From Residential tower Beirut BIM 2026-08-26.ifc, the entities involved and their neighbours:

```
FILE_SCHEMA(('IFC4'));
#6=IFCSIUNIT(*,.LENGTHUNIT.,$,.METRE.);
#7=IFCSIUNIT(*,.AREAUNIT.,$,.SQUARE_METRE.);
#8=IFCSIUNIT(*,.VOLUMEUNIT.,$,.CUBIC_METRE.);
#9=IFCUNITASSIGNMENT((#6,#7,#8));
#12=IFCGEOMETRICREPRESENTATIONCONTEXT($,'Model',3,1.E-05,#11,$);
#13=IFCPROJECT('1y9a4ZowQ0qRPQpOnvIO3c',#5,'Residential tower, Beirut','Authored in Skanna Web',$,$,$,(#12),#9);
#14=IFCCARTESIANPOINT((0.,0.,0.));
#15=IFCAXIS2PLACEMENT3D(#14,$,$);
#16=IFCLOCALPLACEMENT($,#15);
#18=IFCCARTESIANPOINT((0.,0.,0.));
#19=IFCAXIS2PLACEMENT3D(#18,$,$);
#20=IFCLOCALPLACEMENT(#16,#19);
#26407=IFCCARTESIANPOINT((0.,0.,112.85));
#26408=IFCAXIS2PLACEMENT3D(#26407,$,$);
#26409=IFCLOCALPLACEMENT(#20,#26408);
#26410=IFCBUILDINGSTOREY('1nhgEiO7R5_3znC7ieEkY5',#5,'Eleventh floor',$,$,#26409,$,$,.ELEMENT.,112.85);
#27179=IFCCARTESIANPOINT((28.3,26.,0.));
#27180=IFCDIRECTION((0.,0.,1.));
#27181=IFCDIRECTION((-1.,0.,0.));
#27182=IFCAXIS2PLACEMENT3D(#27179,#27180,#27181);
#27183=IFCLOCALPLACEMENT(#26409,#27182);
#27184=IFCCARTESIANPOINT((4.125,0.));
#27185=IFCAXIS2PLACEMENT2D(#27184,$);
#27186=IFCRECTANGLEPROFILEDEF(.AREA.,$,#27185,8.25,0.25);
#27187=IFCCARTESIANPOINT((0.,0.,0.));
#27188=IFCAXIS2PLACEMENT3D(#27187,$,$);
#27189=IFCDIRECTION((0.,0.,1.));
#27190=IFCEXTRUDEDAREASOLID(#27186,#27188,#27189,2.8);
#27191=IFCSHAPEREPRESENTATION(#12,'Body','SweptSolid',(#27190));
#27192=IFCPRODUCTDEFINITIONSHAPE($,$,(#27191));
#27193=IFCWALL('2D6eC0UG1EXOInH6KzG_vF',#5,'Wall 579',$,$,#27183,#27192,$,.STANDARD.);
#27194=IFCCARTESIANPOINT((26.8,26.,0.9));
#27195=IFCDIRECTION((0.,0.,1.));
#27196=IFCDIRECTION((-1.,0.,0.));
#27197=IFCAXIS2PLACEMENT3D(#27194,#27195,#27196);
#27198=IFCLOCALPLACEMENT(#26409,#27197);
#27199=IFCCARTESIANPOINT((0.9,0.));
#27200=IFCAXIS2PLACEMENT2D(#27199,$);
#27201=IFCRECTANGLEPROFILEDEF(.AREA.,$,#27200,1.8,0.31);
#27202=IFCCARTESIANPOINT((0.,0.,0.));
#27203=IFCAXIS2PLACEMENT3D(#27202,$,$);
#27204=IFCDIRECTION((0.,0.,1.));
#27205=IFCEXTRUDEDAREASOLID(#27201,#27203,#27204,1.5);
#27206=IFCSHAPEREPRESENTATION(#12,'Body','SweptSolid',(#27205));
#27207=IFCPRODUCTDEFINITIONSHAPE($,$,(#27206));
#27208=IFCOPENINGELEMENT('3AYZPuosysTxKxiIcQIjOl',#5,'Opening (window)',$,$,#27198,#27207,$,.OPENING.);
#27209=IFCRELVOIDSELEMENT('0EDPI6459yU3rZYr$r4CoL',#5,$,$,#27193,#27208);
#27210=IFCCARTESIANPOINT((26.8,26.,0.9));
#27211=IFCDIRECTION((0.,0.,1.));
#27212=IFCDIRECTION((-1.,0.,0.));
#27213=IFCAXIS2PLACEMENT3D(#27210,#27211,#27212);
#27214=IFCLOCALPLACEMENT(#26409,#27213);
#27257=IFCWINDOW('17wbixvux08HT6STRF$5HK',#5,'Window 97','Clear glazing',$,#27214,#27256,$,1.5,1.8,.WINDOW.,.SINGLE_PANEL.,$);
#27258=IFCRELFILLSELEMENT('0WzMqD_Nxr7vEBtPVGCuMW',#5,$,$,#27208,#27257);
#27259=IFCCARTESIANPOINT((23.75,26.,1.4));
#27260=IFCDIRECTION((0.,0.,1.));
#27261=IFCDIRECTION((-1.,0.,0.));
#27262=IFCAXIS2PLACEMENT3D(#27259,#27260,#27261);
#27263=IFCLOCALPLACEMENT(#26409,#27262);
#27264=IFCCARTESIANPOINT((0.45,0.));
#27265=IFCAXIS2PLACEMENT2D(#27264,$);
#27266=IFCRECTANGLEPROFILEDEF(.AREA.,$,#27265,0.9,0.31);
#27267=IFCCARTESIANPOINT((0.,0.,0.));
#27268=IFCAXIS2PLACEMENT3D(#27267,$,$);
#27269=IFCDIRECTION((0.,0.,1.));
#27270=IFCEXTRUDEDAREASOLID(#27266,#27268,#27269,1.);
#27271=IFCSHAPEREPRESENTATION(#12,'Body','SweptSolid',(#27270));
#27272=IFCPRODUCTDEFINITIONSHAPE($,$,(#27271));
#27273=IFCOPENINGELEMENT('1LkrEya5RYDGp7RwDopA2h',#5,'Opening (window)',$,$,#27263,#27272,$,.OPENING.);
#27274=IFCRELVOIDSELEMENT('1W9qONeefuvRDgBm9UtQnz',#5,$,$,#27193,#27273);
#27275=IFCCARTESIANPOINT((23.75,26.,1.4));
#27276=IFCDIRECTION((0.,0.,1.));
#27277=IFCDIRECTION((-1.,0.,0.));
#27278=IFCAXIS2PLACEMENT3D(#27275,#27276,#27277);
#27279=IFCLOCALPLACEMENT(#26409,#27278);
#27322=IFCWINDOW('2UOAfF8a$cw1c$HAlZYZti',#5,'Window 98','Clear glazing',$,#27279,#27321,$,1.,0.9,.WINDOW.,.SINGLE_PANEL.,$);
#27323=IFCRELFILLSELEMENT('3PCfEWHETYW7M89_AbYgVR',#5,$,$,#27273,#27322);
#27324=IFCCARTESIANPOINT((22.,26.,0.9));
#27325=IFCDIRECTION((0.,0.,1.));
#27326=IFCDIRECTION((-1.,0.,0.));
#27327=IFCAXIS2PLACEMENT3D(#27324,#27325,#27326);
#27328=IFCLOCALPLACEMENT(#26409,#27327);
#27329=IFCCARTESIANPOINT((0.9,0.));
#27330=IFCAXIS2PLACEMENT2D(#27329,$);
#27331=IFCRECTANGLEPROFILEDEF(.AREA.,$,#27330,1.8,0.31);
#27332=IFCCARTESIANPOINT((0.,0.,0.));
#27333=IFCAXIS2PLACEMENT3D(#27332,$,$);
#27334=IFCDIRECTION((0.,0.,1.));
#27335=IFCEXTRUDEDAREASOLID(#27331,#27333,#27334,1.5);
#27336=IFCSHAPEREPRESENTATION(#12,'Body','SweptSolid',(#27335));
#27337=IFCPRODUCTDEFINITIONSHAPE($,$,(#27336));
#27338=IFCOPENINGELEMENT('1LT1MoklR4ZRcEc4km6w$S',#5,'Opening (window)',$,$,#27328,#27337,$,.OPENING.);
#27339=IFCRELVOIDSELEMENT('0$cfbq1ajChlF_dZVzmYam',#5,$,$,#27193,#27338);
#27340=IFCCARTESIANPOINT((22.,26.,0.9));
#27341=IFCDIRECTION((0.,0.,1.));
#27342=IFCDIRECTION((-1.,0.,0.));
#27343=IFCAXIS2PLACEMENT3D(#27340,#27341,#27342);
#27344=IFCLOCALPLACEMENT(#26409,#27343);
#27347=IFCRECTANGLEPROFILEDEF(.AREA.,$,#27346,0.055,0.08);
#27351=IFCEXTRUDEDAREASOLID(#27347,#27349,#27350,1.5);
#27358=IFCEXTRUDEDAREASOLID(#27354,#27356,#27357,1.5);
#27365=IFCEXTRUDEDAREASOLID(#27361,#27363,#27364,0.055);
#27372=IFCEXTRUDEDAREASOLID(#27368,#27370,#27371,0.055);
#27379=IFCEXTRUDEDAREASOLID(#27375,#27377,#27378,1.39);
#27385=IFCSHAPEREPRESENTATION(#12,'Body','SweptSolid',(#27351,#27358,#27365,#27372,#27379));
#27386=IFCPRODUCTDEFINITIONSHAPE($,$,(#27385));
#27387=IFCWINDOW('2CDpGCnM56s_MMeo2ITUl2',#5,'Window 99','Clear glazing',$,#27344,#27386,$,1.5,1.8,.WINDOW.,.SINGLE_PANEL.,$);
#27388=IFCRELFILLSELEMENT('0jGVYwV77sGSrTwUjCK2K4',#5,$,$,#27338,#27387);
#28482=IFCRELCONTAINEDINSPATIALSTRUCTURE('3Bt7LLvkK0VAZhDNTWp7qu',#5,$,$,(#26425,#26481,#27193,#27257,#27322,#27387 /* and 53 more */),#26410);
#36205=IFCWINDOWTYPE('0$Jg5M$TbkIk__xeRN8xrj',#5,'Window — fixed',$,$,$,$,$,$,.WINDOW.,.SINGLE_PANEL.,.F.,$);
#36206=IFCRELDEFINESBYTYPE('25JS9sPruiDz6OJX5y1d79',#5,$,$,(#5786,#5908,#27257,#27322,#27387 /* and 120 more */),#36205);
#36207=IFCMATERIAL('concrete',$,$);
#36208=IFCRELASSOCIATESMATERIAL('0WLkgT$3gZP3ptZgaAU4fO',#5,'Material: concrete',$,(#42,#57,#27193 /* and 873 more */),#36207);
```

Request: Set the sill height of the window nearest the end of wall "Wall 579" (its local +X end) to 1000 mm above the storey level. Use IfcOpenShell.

```python
import numpy as np
import ifcopenshell
import ifcopenshell.api.geometry
import ifcopenshell.geom
import ifcopenshell.util.element
import ifcopenshell.util.placement
import ifcopenshell.util.shape
import ifcopenshell.util.unit

model = ifcopenshell.open("Residential tower Beirut BIM 2026-08-26.ifc")
unit_scale = ifcopenshell.util.unit.calculate_unit_scale(model)

window = model.by_id(27387)
opening = window.FillsVoids[0].RelatingOpeningElement
storey = ifcopenshell.util.element.get_container(window, ifc_class="IfcBuildingStorey")
level = ifcopenshell.util.placement.get_local_placement(storey.ObjectPlacement)[2, 3]

# The opening's origin need not be at the sill, so measure its lowest point.
shape = ifcopenshell.geom.create_shape(ifcopenshell.geom.settings(), opening)
bottom = ifcopenshell.util.shape.get_shape_bottom_elevation(shape, shape.geometry) / unit_scale
dz = level + 1.0 - bottom

shift = np.array([0.0, 0.0, dz])
# The window is not placed relative to its opening, so move both.
for product in (opening, window):
    matrix = ifcopenshell.util.placement.get_local_placement(product.ObjectPlacement)
    matrix[:3, 3] += shift
    ifcopenshell.api.geometry.edit_object_placement(model, product=product, matrix=matrix, is_si=False)

print(f"moved by {dz * unit_scale:+.3f} m")

model.write("Residential tower Beirut BIM 2026-08-26_v2.ifc")
```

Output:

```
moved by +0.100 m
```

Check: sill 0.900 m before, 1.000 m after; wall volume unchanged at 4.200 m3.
